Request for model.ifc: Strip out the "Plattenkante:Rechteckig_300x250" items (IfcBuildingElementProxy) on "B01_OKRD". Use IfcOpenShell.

First a look at what the model holds.

```python
import ifcopenshell
import ifcopenshell.util.element

model = ifcopenshell.open("model.ifc")
print(model.schema)
storey = next(s for s in model.by_type("IfcBuildingStorey") if s.Name == "B01_OKRD")
proxies = [e for e in ifcopenshell.util.element.get_decomposition(storey) if e.is_a("IfcBuildingElementProxy")]
seen = {}
for e in proxies:
    element_type = ifcopenshell.util.element.get_type(e)
    name = element_type.Name if element_type not in (None, e) else None
    seen[name] = seen.get(name, 0) + 1
for name, count in sorted(seen.items(), key=str):
    print(count, "x", name)
```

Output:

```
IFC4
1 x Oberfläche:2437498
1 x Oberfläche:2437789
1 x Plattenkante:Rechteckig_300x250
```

```python
import ifcopenshell
import ifcopenshell.api.root
import ifcopenshell.util.element

model = ifcopenshell.open("model.ifc")

storey = next(s for s in model.by_type("IfcBuildingStorey") if s.Name == "B01_OKRD")
proxies = [e for e in ifcopenshell.util.element.get_decomposition(storey) if e.is_a("IfcBuildingElementProxy")]
targets = [e for e in proxies if (t := ifcopenshell.util.element.get_type(e)) not in (None, e) and t.Name == "Plattenkante:Rechteckig_300x250"]

for e in targets:
    ifcopenshell.api.root.remove_product(model, product=e)
print(len(targets), "removed")

model.write("model_rev.ifc")
```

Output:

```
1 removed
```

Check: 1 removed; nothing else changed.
